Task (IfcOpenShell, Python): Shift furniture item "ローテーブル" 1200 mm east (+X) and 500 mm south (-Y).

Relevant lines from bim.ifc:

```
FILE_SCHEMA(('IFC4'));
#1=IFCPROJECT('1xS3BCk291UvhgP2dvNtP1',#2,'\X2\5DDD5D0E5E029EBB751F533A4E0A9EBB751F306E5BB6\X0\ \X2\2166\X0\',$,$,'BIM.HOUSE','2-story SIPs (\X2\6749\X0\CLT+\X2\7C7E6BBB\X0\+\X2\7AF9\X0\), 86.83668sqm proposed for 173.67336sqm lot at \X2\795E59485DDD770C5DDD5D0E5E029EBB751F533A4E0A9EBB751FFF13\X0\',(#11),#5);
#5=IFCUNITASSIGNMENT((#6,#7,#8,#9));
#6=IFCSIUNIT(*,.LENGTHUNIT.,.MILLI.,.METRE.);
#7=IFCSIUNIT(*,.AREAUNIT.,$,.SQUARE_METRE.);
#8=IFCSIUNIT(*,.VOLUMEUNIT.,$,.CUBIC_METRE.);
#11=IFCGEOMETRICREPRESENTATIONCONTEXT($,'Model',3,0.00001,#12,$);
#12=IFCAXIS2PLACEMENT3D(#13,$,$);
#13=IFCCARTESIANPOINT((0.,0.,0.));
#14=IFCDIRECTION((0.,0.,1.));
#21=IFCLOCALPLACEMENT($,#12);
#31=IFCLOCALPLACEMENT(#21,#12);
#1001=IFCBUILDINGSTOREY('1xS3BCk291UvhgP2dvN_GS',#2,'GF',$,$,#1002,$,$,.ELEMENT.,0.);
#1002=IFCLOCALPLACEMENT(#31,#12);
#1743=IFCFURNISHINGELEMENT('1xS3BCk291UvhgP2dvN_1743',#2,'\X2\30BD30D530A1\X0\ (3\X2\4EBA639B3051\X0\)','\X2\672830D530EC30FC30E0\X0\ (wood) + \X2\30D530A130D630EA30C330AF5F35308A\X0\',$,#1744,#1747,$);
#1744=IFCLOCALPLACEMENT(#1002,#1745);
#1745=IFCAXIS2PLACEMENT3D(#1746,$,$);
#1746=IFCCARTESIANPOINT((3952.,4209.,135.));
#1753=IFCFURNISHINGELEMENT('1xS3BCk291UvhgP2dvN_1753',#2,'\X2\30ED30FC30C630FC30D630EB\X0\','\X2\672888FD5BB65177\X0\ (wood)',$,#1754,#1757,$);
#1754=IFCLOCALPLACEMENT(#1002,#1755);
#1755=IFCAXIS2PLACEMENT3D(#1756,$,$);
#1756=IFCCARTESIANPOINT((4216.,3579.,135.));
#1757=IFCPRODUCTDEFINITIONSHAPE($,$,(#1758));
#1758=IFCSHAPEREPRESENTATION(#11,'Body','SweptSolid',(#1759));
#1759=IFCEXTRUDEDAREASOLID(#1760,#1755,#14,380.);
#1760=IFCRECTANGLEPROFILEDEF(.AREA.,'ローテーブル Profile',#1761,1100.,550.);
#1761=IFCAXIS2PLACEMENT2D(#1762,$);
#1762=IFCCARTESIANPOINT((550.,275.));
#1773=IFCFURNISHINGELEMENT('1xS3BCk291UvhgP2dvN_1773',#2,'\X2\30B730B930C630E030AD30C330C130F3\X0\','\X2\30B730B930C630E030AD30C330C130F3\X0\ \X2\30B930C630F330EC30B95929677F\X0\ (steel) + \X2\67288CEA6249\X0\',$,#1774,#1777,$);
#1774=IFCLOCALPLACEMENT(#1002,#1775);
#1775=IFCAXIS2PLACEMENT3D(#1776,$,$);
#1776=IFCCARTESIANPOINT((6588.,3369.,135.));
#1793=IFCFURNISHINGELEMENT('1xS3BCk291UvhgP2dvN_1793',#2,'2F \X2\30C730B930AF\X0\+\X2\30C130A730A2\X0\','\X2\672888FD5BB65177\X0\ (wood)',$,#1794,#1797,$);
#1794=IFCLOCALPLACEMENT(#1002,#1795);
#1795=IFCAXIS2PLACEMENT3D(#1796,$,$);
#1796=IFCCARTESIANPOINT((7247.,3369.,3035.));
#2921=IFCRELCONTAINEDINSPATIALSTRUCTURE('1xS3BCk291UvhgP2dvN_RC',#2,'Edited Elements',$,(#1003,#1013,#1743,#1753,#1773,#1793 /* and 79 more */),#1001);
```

```python
import ifcopenshell
import ifcopenshell.api.geometry
import ifcopenshell.util.placement

model = ifcopenshell.open("bim.ifc")

item = model.by_guid("1xS3BCk291UvhgP2dvN_1753")
matrix = ifcopenshell.util.placement.get_local_placement(item.ObjectPlacement)
matrix[0, 3] += 1200.0
matrix[1, 3] -= 500.0
ifcopenshell.api.geometry.edit_object_placement(model, product=item, matrix=matrix, is_si=False)

print(ifcopenshell.util.placement.get_local_placement(item.ObjectPlacement).round(3) + 0.0)

model.write("bim-out.ifc")
```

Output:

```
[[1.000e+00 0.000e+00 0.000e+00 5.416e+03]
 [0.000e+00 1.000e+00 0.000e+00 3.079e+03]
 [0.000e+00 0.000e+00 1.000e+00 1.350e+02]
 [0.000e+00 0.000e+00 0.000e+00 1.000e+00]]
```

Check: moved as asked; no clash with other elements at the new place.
